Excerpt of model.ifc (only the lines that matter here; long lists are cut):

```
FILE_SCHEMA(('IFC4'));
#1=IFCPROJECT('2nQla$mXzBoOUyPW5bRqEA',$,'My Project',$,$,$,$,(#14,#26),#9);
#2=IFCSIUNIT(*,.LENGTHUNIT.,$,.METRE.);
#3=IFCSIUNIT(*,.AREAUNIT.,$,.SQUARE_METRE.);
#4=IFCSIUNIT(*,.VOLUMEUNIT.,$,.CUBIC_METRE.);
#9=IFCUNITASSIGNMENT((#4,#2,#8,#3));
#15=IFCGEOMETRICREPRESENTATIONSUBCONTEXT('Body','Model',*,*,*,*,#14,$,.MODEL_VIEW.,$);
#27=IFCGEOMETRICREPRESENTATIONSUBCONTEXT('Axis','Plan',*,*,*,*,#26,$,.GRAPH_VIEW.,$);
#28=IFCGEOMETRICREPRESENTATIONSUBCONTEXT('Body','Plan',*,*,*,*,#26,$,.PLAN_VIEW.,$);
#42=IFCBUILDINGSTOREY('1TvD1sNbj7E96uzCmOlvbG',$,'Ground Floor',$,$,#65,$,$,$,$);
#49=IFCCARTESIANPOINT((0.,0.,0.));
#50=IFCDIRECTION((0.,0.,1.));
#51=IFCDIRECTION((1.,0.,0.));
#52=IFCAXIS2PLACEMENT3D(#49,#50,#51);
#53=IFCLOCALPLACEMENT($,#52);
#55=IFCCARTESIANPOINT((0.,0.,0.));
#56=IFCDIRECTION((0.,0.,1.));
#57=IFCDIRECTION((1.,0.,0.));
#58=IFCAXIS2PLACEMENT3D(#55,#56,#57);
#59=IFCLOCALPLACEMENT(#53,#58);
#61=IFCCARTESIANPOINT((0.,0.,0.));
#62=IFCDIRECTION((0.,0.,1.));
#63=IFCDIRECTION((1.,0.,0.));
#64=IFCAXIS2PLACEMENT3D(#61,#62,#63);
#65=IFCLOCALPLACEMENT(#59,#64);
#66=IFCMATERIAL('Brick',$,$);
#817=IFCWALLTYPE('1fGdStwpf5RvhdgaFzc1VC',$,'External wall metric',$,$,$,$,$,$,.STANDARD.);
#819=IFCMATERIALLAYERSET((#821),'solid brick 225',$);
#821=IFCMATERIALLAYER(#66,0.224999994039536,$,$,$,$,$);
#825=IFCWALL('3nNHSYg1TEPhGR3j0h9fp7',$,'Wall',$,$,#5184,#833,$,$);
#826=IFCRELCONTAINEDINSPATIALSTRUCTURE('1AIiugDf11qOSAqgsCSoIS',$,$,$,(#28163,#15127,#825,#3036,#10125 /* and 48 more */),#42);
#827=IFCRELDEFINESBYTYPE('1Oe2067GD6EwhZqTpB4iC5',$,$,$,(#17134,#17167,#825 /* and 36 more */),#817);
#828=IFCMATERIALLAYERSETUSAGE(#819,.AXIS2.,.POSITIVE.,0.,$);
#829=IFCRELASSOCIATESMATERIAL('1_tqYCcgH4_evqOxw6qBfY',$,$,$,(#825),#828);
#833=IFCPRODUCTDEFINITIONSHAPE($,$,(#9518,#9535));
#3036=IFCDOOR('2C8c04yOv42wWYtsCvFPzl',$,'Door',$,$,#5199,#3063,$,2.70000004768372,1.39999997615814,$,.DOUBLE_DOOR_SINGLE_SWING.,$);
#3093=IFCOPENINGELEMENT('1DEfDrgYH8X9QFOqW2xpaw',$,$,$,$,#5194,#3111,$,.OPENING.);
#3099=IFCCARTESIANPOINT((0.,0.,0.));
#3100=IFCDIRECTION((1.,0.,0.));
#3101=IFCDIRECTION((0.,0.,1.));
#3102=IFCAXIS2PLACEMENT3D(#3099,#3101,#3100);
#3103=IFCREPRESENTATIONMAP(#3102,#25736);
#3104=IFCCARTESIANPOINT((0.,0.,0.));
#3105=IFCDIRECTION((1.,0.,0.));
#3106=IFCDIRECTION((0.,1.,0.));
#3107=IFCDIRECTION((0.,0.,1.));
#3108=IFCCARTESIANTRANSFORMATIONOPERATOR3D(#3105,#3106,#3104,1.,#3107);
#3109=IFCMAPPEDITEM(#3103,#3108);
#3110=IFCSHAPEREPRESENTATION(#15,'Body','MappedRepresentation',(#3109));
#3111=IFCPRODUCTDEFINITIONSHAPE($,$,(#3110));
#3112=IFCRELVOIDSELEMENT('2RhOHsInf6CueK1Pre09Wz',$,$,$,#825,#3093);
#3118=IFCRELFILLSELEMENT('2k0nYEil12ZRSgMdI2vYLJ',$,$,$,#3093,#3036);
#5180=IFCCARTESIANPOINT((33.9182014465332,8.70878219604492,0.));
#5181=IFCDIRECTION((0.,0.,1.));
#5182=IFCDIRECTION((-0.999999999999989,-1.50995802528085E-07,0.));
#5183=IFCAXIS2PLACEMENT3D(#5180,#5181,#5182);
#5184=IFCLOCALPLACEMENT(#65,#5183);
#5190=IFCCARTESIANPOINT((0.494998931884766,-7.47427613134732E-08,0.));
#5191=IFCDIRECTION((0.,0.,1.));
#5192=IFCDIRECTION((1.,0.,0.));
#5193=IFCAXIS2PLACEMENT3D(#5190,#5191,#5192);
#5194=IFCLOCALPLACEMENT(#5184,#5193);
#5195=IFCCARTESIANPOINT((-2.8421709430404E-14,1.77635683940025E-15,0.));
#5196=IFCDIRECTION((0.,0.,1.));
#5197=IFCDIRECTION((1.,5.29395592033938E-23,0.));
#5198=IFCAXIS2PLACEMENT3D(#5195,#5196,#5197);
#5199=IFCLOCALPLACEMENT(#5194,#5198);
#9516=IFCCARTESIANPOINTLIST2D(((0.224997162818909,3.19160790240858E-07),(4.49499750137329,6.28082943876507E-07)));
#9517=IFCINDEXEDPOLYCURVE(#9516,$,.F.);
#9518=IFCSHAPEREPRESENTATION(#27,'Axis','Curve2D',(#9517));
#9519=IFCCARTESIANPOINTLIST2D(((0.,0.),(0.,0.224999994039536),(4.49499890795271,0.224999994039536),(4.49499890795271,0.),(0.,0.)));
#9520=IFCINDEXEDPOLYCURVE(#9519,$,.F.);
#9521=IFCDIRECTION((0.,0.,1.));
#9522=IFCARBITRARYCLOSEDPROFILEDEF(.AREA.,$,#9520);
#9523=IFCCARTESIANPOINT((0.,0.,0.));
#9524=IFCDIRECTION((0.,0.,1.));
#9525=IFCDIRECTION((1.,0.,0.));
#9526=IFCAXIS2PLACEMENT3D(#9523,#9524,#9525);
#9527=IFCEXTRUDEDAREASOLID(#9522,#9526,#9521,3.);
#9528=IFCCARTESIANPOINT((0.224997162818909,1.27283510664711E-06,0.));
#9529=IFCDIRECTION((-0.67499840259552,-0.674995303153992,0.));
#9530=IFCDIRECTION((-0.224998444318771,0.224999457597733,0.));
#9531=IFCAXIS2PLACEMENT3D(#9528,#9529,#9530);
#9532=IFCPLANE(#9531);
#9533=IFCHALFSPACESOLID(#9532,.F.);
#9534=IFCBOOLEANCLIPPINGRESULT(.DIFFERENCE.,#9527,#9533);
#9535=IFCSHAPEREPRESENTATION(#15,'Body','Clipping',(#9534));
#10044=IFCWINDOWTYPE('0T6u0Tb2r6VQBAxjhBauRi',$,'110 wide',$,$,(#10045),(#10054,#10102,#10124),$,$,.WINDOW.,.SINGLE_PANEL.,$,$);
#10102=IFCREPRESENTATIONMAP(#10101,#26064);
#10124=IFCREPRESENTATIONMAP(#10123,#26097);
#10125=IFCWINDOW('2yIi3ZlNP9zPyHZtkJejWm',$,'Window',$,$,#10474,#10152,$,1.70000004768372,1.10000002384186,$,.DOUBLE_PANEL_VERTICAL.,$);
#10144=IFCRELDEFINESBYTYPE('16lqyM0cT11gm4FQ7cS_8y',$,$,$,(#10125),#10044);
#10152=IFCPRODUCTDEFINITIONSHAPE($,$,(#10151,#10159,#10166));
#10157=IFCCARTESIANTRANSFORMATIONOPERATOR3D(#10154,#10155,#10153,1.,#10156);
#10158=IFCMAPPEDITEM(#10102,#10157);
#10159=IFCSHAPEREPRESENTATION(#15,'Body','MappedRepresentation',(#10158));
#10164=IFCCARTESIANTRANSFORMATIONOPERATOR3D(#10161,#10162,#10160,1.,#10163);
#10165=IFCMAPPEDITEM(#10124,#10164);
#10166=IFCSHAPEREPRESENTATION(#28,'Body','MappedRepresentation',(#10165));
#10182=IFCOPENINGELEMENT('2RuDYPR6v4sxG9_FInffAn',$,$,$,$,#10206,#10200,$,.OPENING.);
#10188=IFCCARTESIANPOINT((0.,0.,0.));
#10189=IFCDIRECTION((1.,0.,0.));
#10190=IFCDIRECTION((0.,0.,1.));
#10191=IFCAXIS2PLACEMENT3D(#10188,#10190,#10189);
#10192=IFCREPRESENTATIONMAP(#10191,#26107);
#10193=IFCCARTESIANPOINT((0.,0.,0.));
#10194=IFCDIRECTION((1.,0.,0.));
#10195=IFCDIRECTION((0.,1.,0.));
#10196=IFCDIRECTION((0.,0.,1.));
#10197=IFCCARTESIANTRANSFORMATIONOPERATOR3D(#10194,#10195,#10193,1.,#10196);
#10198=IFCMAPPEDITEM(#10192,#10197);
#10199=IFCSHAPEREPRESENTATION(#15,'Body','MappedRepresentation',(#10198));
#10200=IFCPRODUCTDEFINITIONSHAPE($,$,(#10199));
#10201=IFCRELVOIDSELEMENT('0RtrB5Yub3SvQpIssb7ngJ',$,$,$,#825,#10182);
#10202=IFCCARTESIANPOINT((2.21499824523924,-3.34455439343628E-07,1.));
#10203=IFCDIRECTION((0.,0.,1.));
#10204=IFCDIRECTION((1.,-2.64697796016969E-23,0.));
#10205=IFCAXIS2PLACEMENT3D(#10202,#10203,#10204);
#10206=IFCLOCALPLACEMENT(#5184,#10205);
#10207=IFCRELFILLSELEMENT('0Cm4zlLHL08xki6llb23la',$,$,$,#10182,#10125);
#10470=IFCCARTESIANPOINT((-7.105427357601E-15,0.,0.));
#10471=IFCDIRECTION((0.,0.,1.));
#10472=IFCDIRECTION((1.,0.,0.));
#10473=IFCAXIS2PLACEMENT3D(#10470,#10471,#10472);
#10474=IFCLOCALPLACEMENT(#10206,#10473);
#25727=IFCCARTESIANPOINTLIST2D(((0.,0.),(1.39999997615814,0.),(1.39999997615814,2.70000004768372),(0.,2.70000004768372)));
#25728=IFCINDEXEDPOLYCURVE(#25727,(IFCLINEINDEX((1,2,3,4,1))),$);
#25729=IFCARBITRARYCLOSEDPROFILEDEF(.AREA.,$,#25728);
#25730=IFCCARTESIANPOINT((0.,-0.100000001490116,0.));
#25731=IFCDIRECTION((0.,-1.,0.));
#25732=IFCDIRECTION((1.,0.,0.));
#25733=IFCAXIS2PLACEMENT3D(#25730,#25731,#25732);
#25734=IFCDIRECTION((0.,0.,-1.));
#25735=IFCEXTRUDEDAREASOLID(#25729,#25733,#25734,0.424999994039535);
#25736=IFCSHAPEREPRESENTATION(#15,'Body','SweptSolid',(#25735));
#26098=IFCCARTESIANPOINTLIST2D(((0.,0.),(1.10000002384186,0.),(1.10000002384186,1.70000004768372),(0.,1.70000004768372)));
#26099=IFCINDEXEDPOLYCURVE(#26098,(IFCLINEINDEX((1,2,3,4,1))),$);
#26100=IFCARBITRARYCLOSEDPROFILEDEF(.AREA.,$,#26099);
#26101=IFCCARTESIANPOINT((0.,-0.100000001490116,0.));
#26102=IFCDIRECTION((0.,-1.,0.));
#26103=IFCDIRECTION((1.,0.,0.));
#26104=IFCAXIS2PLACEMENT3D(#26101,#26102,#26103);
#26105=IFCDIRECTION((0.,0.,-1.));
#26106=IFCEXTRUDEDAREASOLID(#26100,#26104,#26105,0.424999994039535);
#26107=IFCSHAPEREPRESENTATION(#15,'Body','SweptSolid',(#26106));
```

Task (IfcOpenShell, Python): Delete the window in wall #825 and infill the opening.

```python
import ifcopenshell
import ifcopenshell.api.feature
import ifcopenshell.api.root
import ifcopenshell.geom
import ifcopenshell.util.shape

model = ifcopenshell.open("model.ifc")
settings = ifcopenshell.geom.settings()


def volume(element):
    """Net volume in cubic metres, openings subtracted."""
    shape = ifcopenshell.geom.create_shape(settings, element)
    return ifcopenshell.util.shape.get_volume(shape.geometry)


window = model.by_id(10125)
opening = window.FillsVoids[0].RelatingOpeningElement
wall = opening.VoidsElements[0].RelatingBuildingElement
before = volume(wall)

ifcopenshell.api.root.remove_product(model, product=window)
ifcopenshell.api.feature.remove_feature(model, feature=opening)

after = volume(wall)

print(f"wall volume {before:.3f} -> {after:.3f} m3")

model.write("model-out.ifc")
```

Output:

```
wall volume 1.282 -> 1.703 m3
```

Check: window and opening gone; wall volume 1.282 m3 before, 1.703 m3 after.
